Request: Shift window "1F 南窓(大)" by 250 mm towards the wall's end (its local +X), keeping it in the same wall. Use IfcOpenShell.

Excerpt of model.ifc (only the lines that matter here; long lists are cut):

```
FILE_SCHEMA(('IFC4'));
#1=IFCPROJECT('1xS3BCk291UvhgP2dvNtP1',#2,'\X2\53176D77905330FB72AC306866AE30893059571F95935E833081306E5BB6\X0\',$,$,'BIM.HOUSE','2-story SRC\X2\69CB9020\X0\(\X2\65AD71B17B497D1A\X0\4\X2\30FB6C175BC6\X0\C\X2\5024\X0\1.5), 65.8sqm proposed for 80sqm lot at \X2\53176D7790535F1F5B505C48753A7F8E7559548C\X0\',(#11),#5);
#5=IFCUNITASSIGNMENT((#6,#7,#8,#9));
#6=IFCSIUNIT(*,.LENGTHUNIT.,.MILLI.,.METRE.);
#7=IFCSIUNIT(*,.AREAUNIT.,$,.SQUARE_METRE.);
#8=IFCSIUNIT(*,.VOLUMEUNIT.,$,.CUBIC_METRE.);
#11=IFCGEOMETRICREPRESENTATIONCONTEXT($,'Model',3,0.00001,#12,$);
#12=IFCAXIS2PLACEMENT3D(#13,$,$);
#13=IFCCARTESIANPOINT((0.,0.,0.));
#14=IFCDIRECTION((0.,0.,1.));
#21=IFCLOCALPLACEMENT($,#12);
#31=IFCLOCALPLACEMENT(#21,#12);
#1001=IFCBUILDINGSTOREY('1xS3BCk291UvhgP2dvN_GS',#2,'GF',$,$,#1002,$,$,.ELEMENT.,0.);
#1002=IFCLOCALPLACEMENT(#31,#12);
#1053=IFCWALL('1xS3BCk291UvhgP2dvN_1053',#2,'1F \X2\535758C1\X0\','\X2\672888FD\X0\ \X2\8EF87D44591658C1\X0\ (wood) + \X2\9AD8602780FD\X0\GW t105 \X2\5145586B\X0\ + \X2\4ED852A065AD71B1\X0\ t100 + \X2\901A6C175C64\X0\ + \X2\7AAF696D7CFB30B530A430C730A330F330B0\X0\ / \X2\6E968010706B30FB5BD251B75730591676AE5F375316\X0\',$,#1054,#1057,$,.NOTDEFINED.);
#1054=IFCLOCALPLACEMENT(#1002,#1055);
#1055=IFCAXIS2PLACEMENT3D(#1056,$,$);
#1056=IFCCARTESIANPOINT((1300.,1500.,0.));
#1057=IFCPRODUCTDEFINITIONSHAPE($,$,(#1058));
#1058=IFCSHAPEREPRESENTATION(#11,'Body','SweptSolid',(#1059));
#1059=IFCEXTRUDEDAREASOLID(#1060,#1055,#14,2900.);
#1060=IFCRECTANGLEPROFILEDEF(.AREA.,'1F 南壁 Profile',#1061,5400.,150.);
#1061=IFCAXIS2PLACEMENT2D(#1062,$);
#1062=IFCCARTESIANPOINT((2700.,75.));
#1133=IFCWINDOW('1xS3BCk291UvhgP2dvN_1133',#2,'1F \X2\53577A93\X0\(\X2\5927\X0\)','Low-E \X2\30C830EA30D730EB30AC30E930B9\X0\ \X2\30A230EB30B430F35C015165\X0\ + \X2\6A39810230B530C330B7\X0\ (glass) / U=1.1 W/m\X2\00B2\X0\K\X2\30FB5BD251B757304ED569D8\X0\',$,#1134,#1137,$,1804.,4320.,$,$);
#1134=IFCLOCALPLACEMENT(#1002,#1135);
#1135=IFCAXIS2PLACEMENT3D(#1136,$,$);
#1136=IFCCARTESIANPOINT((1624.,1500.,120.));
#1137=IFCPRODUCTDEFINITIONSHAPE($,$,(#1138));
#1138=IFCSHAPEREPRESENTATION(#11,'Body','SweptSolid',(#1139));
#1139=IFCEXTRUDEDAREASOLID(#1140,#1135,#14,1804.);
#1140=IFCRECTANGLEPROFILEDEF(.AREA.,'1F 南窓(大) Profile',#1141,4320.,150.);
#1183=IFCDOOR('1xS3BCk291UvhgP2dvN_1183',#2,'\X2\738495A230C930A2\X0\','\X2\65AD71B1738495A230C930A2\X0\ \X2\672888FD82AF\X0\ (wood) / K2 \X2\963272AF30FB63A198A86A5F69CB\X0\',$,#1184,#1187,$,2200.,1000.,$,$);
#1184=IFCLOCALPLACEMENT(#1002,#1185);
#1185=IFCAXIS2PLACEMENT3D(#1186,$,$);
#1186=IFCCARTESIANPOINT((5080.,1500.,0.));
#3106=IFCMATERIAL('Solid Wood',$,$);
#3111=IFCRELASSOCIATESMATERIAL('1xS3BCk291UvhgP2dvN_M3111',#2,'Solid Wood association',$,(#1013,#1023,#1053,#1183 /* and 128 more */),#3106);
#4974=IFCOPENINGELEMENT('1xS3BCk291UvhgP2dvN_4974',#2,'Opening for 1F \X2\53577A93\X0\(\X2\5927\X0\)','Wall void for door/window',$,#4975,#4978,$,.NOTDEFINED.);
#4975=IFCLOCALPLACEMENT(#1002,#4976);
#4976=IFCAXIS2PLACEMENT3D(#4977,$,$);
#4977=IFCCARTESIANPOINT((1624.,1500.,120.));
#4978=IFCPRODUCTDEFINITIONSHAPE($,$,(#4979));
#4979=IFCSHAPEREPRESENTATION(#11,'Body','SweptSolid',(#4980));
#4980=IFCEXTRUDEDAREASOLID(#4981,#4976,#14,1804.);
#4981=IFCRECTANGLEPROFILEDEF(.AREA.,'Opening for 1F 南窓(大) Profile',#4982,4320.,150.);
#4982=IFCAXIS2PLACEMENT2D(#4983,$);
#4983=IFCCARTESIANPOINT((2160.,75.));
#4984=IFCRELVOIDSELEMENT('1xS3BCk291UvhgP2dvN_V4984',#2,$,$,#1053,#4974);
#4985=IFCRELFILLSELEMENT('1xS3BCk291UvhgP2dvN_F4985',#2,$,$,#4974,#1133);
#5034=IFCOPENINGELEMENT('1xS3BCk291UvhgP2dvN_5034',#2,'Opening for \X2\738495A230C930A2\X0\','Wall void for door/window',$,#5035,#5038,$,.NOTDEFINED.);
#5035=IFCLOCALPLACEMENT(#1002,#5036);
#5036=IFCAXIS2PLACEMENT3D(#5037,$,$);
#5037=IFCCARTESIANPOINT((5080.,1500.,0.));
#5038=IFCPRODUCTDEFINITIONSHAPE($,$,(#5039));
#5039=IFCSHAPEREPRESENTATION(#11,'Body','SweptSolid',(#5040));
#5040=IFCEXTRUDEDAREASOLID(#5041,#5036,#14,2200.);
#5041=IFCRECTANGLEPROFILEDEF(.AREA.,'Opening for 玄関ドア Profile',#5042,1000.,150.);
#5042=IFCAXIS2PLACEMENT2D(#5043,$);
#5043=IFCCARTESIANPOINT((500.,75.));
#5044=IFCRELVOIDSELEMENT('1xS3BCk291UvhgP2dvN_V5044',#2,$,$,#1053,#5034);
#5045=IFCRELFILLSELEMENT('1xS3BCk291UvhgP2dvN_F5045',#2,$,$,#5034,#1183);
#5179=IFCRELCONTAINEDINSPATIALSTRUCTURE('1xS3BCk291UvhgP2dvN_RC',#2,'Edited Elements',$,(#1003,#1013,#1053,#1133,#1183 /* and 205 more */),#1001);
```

```python
import ifcopenshell
import ifcopenshell.api.geometry
import ifcopenshell.util.placement
import ifcopenshell.util.unit

model = ifcopenshell.open("model.ifc")
unit_scale = ifcopenshell.util.unit.calculate_unit_scale(model)

window = model.by_guid("1xS3BCk291UvhgP2dvN_1133")
opening = window.FillsVoids[0].RelatingOpeningElement
wall = opening.VoidsElements[0].RelatingBuildingElement

wall_matrix = ifcopenshell.util.placement.get_local_placement(wall.ObjectPlacement)
shift = wall_matrix[:3, 0] * 0.25 / unit_scale
before = ifcopenshell.util.placement.get_local_placement(window.ObjectPlacement)[:3, 3].copy()

# The window is not placed relative to its opening, so move both.
for product in (opening, window):
    matrix = ifcopenshell.util.placement.get_local_placement(product.ObjectPlacement)
    matrix[:3, 3] += shift
    ifcopenshell.api.geometry.edit_object_placement(model, product=product, matrix=matrix, is_si=False)

after = ifcopenshell.util.placement.get_local_placement(window.ObjectPlacement)[:3, 3]
print("window moved by", (after - before).round(3) + 0.0)

model.write("model-out.ifc")
```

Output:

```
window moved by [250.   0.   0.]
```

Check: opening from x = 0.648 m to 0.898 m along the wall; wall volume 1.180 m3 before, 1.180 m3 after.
